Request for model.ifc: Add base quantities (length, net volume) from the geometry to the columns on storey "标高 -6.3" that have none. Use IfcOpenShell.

First a look at what the model holds.

```python
import ifcopenshell
import ifcopenshell.util.element
import ifcopenshell.util.unit

model = ifcopenshell.open("model.ifc")
print(model.schema)
for unit_type in ("LENGTHUNIT", "AREAUNIT", "VOLUMEUNIT"):
    print(unit_type, ifcopenshell.util.unit.calculate_unit_scale(model, unit_type))
storey = next(s for s in model.by_type("IfcBuildingStorey") if s.Name == "标高 -6.3")
columns = [e for e in ifcopenshell.util.element.get_decomposition(storey) if e.is_a("IfcColumn")]
for e in sorted(columns, key=lambda e: e.id()):
    print(e.id(), e.is_a(), e.Name, list(ifcopenshell.util.element.get_psets(e, qtos_only=True)), sep=" | ")
```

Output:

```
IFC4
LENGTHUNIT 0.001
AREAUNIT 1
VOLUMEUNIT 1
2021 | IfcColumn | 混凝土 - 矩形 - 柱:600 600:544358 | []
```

```python
import ifcopenshell
import ifcopenshell.api.pset
import ifcopenshell.geom
import ifcopenshell.util.element
import ifcopenshell.util.shape
import ifcopenshell.util.unit

model = ifcopenshell.open("model.ifc")
unit_scale = ifcopenshell.util.unit.calculate_unit_scale(model)
volume_scale = ifcopenshell.util.unit.calculate_unit_scale(model, "VOLUMEUNIT")
settings = ifcopenshell.geom.settings()

storey = next(s for s in model.by_type("IfcBuildingStorey") if s.Name == "标高 -6.3")
columns = [e for e in ifcopenshell.util.element.get_decomposition(storey) if e.is_a("IfcColumn")]

for e in sorted(columns, key=lambda e: e.id()):
    if ifcopenshell.util.element.get_psets(e, qtos_only=True, should_inherit=False):
        continue
    # Geometry comes back in metres, in the element's own axes.
    shape = ifcopenshell.geom.create_shape(settings, e)
    values = {
        "Length": ifcopenshell.util.shape.get_z(shape.geometry) / unit_scale,
        "NetVolume": ifcopenshell.util.shape.get_volume(shape.geometry) / volume_scale,
    }
    qto = ifcopenshell.api.pset.add_qto(model, product=e, name="Qto_ColumnBaseQuantities")
    ifcopenshell.api.pset.edit_qto(model, qto=qto, properties=values)
    print(e.id(), {k: round(v, 3) for k, v in values.items()})

model.write("model_updated.ifc")
```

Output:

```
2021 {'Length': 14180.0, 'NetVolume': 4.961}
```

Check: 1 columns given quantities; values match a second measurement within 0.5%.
